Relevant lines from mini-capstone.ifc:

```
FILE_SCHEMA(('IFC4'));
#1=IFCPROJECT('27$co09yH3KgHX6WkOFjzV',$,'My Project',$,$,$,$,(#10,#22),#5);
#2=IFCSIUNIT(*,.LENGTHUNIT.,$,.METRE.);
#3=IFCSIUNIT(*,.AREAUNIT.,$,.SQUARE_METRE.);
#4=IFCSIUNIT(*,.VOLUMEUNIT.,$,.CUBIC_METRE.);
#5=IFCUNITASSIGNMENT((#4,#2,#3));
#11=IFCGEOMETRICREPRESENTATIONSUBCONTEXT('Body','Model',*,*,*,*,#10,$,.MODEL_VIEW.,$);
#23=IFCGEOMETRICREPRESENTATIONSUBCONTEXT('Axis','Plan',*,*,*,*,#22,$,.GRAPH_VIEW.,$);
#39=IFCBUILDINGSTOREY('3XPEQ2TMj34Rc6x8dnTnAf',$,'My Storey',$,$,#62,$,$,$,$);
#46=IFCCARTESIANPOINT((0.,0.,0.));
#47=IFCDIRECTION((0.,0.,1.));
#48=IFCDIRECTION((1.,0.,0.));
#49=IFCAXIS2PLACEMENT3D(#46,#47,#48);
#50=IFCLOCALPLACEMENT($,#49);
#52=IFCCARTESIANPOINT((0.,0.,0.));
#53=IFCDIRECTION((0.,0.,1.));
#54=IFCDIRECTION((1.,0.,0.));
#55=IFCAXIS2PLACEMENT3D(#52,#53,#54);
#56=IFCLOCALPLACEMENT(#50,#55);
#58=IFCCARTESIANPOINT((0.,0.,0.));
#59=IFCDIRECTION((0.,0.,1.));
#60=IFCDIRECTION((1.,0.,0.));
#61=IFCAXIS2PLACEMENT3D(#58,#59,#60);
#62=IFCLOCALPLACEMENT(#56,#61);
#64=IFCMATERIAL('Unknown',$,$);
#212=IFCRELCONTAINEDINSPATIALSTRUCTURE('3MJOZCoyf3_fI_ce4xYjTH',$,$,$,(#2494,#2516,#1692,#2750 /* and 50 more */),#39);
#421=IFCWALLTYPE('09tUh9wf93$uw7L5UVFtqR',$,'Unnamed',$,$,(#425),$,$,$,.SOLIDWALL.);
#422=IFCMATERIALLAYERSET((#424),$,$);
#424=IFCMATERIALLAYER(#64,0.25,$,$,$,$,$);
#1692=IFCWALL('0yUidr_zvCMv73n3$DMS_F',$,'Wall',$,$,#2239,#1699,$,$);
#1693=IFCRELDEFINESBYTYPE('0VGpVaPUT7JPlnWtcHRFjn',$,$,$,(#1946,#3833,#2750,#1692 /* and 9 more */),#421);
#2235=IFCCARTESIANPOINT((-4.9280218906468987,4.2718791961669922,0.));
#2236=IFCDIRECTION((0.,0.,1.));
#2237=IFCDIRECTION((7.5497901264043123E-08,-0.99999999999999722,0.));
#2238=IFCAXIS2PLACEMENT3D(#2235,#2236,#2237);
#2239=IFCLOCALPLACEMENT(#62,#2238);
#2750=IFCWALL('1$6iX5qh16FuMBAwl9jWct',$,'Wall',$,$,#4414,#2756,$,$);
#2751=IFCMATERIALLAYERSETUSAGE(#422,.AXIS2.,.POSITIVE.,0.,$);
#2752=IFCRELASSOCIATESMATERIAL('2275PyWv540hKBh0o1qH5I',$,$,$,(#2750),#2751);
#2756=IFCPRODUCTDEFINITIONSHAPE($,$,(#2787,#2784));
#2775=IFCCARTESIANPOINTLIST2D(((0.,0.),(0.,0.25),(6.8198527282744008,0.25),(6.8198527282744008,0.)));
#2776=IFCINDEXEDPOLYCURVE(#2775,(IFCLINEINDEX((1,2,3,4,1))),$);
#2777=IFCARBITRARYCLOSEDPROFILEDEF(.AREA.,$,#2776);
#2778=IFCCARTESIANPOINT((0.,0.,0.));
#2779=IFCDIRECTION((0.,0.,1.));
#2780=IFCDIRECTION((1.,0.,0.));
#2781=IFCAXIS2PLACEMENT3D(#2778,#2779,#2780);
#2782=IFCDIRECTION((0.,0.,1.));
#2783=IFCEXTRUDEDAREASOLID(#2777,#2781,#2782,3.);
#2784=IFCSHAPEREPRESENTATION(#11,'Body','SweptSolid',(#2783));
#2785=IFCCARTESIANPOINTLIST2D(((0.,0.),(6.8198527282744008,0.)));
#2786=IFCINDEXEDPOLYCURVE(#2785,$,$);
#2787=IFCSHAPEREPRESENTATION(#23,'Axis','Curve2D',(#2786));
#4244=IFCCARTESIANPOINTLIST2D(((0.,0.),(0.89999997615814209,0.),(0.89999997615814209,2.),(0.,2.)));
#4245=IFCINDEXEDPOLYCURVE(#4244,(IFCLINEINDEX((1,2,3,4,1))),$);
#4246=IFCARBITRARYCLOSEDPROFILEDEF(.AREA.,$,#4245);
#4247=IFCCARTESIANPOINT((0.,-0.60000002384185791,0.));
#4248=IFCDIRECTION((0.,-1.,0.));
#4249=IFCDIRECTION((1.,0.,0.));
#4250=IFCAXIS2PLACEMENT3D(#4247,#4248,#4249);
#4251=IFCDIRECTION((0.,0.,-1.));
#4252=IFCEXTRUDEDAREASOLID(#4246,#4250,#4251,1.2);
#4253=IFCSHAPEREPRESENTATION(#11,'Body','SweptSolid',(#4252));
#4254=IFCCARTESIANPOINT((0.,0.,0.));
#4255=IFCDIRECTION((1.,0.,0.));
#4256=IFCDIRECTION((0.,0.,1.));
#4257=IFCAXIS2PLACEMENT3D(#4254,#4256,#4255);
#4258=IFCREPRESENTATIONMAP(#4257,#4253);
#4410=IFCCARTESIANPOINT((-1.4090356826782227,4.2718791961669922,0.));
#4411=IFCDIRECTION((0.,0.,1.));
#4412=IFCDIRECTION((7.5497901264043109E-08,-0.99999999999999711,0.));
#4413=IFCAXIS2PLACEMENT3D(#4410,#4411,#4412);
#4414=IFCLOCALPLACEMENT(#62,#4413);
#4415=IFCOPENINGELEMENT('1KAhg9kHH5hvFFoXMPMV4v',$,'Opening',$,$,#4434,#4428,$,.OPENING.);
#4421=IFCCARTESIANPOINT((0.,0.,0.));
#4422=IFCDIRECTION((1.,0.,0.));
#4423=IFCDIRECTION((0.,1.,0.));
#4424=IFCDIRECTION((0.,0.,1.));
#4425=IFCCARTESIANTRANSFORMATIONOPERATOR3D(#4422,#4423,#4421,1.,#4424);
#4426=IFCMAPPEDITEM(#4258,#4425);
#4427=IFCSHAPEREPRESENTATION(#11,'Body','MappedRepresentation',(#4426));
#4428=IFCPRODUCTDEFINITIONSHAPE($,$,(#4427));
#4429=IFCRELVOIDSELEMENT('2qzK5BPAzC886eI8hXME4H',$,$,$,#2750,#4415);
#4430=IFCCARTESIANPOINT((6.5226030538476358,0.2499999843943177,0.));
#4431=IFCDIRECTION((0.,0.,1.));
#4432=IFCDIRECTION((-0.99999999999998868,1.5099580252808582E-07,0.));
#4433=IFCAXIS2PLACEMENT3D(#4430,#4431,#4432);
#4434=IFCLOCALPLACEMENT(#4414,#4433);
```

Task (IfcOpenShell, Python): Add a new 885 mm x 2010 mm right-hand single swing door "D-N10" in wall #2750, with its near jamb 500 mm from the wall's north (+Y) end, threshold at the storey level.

```python
import numpy as np
import ifcopenshell
import ifcopenshell.api.feature
import ifcopenshell.api.geometry
import ifcopenshell.api.root
import ifcopenshell.api.spatial
import ifcopenshell.geom
import ifcopenshell.util.element
import ifcopenshell.util.placement
import ifcopenshell.util.representation
import ifcopenshell.util.shape
import ifcopenshell.util.unit

model = ifcopenshell.open("mini-capstone.ifc")
unit_scale = ifcopenshell.util.unit.calculate_unit_scale(model)
settings = ifcopenshell.geom.settings()


def volume(element):
    """Net volume in cubic metres, openings subtracted."""
    shape = ifcopenshell.geom.create_shape(settings, element)
    return ifcopenshell.util.shape.get_volume(shape.geometry)


wall = model.by_id(2750)
storey = ifcopenshell.util.element.get_container(wall, ifc_class="IfcBuildingStorey")
context = ifcopenshell.util.representation.get_context(model, "Model", "Body", "MODEL_VIEW")
before = volume(wall)

width, height, from_end, sill = 0.885, 2.01, 0.5, 0.0  # metres

# The wall runs along its own X axis, and the end named is its -X end.
wall_shape = ifcopenshell.geom.create_shape(settings, wall)
x, y, z = ifcopenshell.util.shape.get_vertices(wall_shape.geometry).T
start = x.min() + from_end
face, thickness = float(y.min()), float(y.max() - y.min())
wall_matrix = ifcopenshell.util.placement.get_local_placement(wall.ObjectPlacement)
level = ifcopenshell.util.placement.get_local_placement(storey.ObjectPlacement)[2, 3]


def in_wall(x, y):
    """Placement at x, y metres in the wall's axes, at sill height."""
    matrix = wall_matrix.copy()
    matrix[:, 3] = wall_matrix @ np.array([x / unit_scale, y / unit_scale, 0.0, 1.0])
    matrix[2, 3] = level + sill / unit_scale
    return matrix


# Opening: a box that overshoots both wall faces by 50 mm.
opening = ifcopenshell.api.root.create_entity(model, ifc_class="IfcOpeningElement", predefined_type="OPENING")
box = ifcopenshell.api.geometry.add_wall_representation(
    model, context=context, length=width, height=height, thickness=thickness + 0.1
)
ifcopenshell.api.geometry.assign_representation(model, product=opening, representation=box)
ifcopenshell.api.geometry.edit_object_placement(model, product=opening, matrix=in_wall(start, face - 0.05), is_si=False)
ifcopenshell.api.feature.add_feature(model, feature=opening, element=wall)

door = ifcopenshell.api.root.create_entity(model, ifc_class="IfcDoor", name="D-N10", predefined_type="DOOR")
door.OverallWidth, door.OverallHeight = width / unit_scale, height / unit_scale
door.OperationType = "SINGLE_SWING_RIGHT"
body = ifcopenshell.api.geometry.add_door_representation(
    model,
    context=context,
    overall_width=door.OverallWidth,
    overall_height=door.OverallHeight,
    operation_type="SINGLE_SWING_RIGHT",
    lining_properties={"LiningDepth": thickness / unit_scale, "ThresholdDepth": thickness / unit_scale},
)
ifcopenshell.api.geometry.assign_representation(model, product=door, representation=body)
ifcopenshell.api.spatial.assign_container(model, products=[door], relating_structure=storey)
ifcopenshell.api.feature.add_filling(model, opening=opening, element=door)

# The lining spans the wall, so the door starts at the wall face.
ifcopenshell.api.geometry.edit_object_placement(model, product=door, matrix=in_wall(start, face), is_si=False)

after = volume(wall)

print(f"wall volume {before:.3f} -> {after:.3f} m3")

model.write("mini-capstone_edited.ifc")
```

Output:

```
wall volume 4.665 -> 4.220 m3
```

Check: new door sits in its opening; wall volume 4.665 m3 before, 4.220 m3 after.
